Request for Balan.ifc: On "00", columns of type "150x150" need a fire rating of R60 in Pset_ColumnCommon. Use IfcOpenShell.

First a look at what the model holds.

```python
import ifcopenshell
import ifcopenshell.util.element

model = ifcopenshell.open("Balan.ifc")
print(model.schema)
storey = next(s for s in model.by_type("IfcBuildingStorey") if s.Name == "00")
columns = [e for e in ifcopenshell.util.element.get_decomposition(storey) if e.is_a("IfcColumn")]
seen = {}
for e in columns:
    element_type = ifcopenshell.util.element.get_type(e)
    key = (element_type.Name if element_type != e and element_type else None, ifcopenshell.util.element.get_pset(e, "Pset_ColumnCommon", "FireRating"))
    seen[key] = seen.get(key, 0) + 1
for (name, value), count in sorted(seen.items(), key=str):
    print(count, "x", name, "|", value)
```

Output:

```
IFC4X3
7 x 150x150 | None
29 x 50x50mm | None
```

```python
import ifcopenshell
import ifcopenshell.api.pset
import ifcopenshell.util.element

model = ifcopenshell.open("Balan.ifc")

storey = next(s for s in model.by_type("IfcBuildingStorey") if s.Name == "00")
columns = [e for e in ifcopenshell.util.element.get_decomposition(storey) if e.is_a("IfcColumn")]

count = 0
for e in columns:
    element_type = ifcopenshell.util.element.get_type(e)
    if element_type in (None, e) or element_type.Name != "150x150":
        continue
    # add_pset returns the element's existing set when there is one.
    pset = ifcopenshell.api.pset.add_pset(model, product=e, name="Pset_ColumnCommon")
    ifcopenshell.api.pset.edit_pset(model, pset=pset, properties={"FireRating": "R60"})
    count += 1

print(count, "columns updated")

model.write("Balan-out.ifc")
```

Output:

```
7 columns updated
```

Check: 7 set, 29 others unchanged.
